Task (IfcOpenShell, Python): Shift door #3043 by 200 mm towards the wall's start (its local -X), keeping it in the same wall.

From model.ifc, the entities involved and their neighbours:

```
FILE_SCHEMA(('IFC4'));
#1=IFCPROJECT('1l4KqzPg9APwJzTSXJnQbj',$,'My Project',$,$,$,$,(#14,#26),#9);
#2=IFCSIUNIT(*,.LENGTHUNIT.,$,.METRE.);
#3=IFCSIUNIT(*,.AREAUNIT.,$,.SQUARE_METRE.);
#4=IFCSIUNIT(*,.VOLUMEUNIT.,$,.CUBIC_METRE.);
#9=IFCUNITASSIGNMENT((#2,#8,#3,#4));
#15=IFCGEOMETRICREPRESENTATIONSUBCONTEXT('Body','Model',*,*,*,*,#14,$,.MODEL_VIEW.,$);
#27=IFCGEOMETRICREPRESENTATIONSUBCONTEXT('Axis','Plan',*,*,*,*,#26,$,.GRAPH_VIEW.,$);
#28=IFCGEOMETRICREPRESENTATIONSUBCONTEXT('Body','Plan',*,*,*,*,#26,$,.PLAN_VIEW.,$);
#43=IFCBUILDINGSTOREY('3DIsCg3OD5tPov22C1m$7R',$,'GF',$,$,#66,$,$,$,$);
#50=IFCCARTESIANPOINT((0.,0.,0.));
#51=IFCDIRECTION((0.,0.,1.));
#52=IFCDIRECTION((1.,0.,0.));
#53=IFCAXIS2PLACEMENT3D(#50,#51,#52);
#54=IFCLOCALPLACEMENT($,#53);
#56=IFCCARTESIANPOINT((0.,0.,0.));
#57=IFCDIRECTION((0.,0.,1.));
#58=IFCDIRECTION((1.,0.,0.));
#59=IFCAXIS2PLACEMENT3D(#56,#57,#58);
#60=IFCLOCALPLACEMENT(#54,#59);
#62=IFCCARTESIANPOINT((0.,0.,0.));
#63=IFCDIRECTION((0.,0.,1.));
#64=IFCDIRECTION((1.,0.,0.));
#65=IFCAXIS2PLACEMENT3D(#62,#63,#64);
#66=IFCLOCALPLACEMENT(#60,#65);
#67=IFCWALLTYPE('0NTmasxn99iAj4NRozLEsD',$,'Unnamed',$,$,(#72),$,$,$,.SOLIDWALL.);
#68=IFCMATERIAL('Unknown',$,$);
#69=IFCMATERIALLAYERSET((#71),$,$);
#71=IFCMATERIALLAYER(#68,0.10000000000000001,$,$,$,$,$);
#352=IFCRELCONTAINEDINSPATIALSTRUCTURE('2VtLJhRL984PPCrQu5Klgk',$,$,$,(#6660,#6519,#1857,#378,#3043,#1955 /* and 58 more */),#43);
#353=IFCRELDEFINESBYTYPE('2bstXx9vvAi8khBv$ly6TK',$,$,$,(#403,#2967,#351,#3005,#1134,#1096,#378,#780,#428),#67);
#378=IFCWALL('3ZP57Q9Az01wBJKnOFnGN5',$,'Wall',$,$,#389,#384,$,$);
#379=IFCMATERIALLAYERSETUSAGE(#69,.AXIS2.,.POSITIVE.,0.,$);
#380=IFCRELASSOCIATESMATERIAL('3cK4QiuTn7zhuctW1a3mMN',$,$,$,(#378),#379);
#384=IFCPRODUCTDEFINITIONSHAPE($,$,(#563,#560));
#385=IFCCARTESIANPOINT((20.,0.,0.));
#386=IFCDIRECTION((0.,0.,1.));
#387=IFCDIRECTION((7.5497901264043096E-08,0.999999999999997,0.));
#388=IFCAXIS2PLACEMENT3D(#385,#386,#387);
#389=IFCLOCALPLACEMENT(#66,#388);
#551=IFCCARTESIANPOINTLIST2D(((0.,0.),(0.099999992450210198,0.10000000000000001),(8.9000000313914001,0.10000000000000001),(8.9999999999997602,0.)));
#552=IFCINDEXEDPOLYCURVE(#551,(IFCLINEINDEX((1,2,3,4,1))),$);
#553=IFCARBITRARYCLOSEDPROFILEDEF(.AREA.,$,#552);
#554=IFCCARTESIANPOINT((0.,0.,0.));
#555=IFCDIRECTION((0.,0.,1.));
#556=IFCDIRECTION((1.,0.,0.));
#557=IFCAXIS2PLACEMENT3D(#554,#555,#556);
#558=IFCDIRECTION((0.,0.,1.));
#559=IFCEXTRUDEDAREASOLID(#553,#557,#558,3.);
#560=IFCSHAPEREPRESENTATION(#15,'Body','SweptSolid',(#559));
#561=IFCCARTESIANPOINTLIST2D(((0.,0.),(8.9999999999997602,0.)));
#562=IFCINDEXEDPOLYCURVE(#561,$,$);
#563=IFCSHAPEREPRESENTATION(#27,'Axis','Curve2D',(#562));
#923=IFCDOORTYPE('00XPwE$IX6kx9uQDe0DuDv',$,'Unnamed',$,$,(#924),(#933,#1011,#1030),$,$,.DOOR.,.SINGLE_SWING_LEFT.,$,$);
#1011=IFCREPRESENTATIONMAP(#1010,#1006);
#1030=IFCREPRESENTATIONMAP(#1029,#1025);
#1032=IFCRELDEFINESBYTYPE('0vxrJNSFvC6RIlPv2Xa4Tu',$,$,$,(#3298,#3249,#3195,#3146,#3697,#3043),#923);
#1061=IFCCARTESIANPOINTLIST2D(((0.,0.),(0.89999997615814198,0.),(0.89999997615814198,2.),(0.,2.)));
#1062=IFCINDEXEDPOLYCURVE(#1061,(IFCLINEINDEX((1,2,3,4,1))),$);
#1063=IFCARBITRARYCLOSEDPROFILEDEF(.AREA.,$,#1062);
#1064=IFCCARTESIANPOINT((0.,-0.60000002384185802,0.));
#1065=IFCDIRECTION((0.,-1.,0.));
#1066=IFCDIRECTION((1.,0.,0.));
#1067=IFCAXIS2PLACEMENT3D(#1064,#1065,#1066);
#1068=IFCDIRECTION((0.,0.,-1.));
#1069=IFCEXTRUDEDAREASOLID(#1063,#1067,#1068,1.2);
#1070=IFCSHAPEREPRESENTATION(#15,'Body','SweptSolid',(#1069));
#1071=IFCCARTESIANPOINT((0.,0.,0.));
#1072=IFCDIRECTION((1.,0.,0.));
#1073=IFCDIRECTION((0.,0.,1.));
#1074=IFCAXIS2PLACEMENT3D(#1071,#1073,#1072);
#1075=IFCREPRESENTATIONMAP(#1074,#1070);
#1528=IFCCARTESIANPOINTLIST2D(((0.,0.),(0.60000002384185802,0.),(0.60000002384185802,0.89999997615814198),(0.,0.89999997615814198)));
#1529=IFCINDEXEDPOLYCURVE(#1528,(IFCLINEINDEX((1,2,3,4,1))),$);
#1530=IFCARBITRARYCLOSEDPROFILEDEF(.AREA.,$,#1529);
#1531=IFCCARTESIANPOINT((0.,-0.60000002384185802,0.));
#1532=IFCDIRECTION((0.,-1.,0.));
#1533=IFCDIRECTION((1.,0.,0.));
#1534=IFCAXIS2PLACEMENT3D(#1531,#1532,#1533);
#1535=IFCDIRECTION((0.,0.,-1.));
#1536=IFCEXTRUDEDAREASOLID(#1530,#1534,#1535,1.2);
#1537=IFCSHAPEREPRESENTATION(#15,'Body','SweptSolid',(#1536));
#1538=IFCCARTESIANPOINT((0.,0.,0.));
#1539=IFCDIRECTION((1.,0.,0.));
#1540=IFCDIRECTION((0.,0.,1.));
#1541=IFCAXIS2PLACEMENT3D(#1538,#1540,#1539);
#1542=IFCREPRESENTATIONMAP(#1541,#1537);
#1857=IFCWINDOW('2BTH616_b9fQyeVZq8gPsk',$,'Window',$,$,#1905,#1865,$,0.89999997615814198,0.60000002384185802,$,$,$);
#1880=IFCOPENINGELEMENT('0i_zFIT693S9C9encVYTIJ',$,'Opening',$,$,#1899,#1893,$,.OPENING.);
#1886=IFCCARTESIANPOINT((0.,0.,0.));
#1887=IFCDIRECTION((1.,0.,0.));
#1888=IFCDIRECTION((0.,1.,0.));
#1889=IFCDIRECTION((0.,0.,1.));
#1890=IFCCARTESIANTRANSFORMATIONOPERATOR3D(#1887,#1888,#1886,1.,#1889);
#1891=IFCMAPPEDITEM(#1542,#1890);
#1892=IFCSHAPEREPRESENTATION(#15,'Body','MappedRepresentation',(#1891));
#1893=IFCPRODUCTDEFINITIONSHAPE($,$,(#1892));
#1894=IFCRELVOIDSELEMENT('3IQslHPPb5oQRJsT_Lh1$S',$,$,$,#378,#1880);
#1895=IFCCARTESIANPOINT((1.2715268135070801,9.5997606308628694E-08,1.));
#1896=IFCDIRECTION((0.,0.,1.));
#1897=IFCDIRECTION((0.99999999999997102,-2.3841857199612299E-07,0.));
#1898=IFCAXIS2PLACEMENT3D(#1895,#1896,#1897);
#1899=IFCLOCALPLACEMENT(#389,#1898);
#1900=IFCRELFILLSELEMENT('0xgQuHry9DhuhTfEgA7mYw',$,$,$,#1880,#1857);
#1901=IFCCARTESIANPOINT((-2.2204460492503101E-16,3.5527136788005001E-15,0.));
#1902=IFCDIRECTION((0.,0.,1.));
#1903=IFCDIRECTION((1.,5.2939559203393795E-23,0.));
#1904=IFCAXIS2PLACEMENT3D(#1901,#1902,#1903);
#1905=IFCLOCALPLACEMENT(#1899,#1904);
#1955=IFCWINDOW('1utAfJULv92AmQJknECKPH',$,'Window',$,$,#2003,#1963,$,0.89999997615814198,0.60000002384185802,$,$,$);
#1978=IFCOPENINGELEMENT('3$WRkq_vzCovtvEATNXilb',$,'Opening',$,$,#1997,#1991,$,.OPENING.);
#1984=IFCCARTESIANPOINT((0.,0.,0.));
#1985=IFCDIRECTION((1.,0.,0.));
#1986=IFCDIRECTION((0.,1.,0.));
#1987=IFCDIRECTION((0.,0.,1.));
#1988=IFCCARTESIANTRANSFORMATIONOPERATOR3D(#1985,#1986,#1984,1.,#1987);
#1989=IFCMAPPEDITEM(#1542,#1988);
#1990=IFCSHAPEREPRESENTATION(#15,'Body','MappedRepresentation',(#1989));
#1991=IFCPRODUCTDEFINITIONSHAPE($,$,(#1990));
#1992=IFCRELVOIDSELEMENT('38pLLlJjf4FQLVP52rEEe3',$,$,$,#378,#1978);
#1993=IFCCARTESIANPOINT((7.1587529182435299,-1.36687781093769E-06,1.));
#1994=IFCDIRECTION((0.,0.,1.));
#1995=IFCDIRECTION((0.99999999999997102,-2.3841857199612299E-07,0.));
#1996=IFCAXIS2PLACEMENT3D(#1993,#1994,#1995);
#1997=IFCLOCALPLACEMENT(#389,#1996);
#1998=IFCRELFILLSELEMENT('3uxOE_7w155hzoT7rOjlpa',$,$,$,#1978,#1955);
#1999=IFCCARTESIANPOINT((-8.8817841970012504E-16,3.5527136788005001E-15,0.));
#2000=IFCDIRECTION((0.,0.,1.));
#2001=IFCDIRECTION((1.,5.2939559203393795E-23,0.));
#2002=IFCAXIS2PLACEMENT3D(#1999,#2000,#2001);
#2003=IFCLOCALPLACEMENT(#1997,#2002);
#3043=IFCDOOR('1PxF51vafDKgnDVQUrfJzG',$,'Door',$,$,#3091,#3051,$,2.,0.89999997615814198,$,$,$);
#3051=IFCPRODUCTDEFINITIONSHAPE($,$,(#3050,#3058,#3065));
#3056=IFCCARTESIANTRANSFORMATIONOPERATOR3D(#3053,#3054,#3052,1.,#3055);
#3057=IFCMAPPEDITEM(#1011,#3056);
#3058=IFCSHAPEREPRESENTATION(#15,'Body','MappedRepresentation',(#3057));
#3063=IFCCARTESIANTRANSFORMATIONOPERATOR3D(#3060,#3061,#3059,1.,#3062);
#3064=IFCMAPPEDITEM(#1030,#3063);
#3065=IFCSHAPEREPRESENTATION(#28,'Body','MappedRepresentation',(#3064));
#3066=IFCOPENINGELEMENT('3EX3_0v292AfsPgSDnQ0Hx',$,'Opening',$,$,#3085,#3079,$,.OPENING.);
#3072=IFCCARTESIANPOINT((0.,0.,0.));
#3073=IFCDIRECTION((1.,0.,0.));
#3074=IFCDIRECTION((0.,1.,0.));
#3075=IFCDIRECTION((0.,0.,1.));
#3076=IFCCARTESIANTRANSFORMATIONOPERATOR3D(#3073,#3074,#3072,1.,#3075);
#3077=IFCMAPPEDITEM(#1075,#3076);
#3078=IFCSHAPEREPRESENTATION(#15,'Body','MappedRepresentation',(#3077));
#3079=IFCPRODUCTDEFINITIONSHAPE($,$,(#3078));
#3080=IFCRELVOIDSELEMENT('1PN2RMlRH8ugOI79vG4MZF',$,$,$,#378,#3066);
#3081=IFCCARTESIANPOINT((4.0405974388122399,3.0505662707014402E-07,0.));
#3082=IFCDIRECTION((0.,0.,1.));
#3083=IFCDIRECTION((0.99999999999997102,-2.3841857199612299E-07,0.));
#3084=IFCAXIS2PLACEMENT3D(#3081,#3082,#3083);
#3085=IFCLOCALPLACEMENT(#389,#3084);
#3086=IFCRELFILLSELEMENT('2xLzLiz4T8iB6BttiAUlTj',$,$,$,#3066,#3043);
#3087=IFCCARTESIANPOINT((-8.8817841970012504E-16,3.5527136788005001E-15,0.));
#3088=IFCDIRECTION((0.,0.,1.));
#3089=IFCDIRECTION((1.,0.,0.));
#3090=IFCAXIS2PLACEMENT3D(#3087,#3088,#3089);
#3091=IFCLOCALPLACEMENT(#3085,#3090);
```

```python
import ifcopenshell
import ifcopenshell.api.geometry
import ifcopenshell.util.placement
import ifcopenshell.util.unit

model = ifcopenshell.open("model.ifc")
unit_scale = ifcopenshell.util.unit.calculate_unit_scale(model)

door = model.by_guid("1PxF51vafDKgnDVQUrfJzG")
opening = door.FillsVoids[0].RelatingOpeningElement
wall = opening.VoidsElements[0].RelatingBuildingElement

wall_matrix = ifcopenshell.util.placement.get_local_placement(wall.ObjectPlacement)
shift = wall_matrix[:3, 0] * -0.2 / unit_scale
before = ifcopenshell.util.placement.get_local_placement(door.ObjectPlacement)[:3, 3].copy()

# The door is placed relative to its opening, so it follows when the opening moves.
matrix = ifcopenshell.util.placement.get_local_placement(opening.ObjectPlacement)
matrix[:3, 3] += shift
ifcopenshell.api.geometry.edit_object_placement(
    model, product=opening, matrix=matrix, is_si=False, should_transform_children=True
)

after = ifcopenshell.util.placement.get_local_placement(door.ObjectPlacement)[:3, 3]
print("door moved by", (after - before).round(3) + 0.0)

model.write("model_v2.ifc")
```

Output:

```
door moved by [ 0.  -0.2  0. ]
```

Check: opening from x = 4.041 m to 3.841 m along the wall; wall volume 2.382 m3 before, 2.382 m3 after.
